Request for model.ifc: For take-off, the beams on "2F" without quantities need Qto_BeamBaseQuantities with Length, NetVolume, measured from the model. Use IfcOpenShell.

First a look at what the model holds.

```python
import ifcopenshell
import ifcopenshell.util.element
import ifcopenshell.util.unit

model = ifcopenshell.open("model.ifc")
print(model.schema)
for unit_type in ("LENGTHUNIT", "AREAUNIT", "VOLUMEUNIT"):
    print(unit_type, ifcopenshell.util.unit.calculate_unit_scale(model, unit_type))
storey = next(s for s in model.by_type("IfcBuildingStorey") if s.Name == "2F")
beams = [e for e in ifcopenshell.util.element.get_decomposition(storey) if e.is_a("IfcBeam")]
for e in sorted(beams, key=lambda e: e.id()):
    print(e.id(), e.is_a(), e.Name, list(ifcopenshell.util.element.get_psets(e, qtos_only=True)), sep=" | ")
```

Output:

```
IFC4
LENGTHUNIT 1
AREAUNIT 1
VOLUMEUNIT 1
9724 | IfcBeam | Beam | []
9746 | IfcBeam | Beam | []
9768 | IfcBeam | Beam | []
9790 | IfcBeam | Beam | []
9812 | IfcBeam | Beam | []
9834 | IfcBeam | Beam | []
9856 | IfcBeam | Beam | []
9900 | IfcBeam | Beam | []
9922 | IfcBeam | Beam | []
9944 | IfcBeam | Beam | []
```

```python
import ifcopenshell
import ifcopenshell.api.pset
import ifcopenshell.geom
import ifcopenshell.util.element
import ifcopenshell.util.shape
import ifcopenshell.util.unit

model = ifcopenshell.open("model.ifc")
unit_scale = ifcopenshell.util.unit.calculate_unit_scale(model)
volume_scale = ifcopenshell.util.unit.calculate_unit_scale(model, "VOLUMEUNIT")
settings = ifcopenshell.geom.settings()

storey = next(s for s in model.by_type("IfcBuildingStorey") if s.Name == "2F")
beams = [e for e in ifcopenshell.util.element.get_decomposition(storey) if e.is_a("IfcBeam")]

for e in sorted(beams, key=lambda e: e.id()):
    if ifcopenshell.util.element.get_psets(e, qtos_only=True, should_inherit=False):
        continue
    # Geometry comes back in metres, in the element's own axes.
    shape = ifcopenshell.geom.create_shape(settings, e)
    values = {
        "Length": ifcopenshell.util.shape.get_max_xyz(shape.geometry) / unit_scale,
        "NetVolume": ifcopenshell.util.shape.get_volume(shape.geometry) / volume_scale,
    }
    qto = ifcopenshell.api.pset.add_qto(model, product=e, name="Qto_BeamBaseQuantities")
    ifcopenshell.api.pset.edit_qto(model, qto=qto, properties=values)
    print(e.id(), {k: round(v, 3) for k, v in values.items()})

model.write("model_v2.ifc")
```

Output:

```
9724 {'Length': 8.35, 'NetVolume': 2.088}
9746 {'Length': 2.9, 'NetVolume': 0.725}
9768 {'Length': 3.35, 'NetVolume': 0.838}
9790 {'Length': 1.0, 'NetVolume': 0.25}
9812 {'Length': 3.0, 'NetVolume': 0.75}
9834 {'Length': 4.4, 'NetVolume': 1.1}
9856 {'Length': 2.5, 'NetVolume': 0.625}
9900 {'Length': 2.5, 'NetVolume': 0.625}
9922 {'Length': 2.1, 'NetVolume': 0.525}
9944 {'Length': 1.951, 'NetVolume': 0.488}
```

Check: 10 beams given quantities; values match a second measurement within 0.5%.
